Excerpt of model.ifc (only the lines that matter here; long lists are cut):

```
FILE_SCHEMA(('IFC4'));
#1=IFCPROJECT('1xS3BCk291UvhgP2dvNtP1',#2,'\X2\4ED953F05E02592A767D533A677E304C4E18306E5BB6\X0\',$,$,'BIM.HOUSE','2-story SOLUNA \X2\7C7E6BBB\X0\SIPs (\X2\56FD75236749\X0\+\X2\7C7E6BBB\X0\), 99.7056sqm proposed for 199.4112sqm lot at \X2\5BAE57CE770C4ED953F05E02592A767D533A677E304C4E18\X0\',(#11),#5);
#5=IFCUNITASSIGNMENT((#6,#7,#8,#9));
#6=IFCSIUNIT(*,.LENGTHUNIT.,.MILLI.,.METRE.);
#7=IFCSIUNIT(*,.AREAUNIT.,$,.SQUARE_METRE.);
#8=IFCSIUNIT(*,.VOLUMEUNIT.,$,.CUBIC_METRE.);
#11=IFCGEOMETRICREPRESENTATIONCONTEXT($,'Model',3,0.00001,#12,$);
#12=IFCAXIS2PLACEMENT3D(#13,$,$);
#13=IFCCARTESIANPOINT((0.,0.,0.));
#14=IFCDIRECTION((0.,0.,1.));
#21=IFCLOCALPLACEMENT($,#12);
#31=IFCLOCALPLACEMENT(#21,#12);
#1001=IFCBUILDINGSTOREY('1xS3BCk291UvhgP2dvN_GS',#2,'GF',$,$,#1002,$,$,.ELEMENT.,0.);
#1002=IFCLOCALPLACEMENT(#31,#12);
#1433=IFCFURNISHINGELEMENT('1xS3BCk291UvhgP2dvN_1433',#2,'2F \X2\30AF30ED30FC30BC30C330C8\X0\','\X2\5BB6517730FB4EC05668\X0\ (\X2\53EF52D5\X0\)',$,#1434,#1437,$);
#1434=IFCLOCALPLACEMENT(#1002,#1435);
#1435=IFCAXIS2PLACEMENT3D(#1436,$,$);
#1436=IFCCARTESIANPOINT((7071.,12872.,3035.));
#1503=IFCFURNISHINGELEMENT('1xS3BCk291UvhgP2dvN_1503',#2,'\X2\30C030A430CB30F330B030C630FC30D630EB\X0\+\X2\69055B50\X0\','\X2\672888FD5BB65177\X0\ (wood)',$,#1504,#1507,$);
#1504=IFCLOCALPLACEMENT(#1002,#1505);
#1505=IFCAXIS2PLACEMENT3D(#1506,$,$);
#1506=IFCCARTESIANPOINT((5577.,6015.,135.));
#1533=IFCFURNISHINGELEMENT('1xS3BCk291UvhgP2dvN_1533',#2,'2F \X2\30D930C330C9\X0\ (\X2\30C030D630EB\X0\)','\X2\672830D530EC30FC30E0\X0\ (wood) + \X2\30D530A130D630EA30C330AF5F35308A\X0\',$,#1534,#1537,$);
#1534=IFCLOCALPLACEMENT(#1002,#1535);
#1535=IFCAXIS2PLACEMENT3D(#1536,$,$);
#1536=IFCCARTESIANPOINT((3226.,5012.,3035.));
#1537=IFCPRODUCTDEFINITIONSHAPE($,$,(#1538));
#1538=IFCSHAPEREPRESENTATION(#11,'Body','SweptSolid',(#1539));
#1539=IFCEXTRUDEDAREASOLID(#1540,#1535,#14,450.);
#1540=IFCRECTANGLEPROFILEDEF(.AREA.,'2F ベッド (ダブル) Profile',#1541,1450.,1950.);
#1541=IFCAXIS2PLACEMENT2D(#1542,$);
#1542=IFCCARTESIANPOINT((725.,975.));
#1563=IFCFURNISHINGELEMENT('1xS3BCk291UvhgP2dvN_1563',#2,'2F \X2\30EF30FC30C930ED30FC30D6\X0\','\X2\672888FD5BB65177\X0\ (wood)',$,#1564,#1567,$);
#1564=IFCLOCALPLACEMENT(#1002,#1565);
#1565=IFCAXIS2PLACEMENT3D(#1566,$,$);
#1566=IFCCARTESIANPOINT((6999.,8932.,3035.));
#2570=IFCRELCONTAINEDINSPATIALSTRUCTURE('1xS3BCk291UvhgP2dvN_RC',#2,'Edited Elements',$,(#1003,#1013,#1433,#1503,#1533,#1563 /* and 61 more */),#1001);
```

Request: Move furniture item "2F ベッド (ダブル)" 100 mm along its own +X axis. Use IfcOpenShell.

```python
import ifcopenshell
import ifcopenshell.api.geometry
import ifcopenshell.util.placement
import ifcopenshell.util.unit

model = ifcopenshell.open("model.ifc")
unit_scale = ifcopenshell.util.unit.calculate_unit_scale(model)

item = model.by_guid("1xS3BCk291UvhgP2dvN_1533")
matrix = ifcopenshell.util.placement.get_local_placement(item.ObjectPlacement)
matrix[:3, 3] += matrix[:3, 0] * 0.1 / unit_scale
ifcopenshell.api.geometry.edit_object_placement(model, product=item, matrix=matrix, is_si=False)

print(ifcopenshell.util.placement.get_local_placement(item.ObjectPlacement).round(3) + 0.0)

model.write("model_edited.ifc")
```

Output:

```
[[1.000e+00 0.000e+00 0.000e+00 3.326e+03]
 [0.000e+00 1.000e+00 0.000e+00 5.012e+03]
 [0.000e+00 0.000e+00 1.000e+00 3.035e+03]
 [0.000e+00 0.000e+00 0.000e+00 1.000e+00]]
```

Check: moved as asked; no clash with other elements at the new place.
